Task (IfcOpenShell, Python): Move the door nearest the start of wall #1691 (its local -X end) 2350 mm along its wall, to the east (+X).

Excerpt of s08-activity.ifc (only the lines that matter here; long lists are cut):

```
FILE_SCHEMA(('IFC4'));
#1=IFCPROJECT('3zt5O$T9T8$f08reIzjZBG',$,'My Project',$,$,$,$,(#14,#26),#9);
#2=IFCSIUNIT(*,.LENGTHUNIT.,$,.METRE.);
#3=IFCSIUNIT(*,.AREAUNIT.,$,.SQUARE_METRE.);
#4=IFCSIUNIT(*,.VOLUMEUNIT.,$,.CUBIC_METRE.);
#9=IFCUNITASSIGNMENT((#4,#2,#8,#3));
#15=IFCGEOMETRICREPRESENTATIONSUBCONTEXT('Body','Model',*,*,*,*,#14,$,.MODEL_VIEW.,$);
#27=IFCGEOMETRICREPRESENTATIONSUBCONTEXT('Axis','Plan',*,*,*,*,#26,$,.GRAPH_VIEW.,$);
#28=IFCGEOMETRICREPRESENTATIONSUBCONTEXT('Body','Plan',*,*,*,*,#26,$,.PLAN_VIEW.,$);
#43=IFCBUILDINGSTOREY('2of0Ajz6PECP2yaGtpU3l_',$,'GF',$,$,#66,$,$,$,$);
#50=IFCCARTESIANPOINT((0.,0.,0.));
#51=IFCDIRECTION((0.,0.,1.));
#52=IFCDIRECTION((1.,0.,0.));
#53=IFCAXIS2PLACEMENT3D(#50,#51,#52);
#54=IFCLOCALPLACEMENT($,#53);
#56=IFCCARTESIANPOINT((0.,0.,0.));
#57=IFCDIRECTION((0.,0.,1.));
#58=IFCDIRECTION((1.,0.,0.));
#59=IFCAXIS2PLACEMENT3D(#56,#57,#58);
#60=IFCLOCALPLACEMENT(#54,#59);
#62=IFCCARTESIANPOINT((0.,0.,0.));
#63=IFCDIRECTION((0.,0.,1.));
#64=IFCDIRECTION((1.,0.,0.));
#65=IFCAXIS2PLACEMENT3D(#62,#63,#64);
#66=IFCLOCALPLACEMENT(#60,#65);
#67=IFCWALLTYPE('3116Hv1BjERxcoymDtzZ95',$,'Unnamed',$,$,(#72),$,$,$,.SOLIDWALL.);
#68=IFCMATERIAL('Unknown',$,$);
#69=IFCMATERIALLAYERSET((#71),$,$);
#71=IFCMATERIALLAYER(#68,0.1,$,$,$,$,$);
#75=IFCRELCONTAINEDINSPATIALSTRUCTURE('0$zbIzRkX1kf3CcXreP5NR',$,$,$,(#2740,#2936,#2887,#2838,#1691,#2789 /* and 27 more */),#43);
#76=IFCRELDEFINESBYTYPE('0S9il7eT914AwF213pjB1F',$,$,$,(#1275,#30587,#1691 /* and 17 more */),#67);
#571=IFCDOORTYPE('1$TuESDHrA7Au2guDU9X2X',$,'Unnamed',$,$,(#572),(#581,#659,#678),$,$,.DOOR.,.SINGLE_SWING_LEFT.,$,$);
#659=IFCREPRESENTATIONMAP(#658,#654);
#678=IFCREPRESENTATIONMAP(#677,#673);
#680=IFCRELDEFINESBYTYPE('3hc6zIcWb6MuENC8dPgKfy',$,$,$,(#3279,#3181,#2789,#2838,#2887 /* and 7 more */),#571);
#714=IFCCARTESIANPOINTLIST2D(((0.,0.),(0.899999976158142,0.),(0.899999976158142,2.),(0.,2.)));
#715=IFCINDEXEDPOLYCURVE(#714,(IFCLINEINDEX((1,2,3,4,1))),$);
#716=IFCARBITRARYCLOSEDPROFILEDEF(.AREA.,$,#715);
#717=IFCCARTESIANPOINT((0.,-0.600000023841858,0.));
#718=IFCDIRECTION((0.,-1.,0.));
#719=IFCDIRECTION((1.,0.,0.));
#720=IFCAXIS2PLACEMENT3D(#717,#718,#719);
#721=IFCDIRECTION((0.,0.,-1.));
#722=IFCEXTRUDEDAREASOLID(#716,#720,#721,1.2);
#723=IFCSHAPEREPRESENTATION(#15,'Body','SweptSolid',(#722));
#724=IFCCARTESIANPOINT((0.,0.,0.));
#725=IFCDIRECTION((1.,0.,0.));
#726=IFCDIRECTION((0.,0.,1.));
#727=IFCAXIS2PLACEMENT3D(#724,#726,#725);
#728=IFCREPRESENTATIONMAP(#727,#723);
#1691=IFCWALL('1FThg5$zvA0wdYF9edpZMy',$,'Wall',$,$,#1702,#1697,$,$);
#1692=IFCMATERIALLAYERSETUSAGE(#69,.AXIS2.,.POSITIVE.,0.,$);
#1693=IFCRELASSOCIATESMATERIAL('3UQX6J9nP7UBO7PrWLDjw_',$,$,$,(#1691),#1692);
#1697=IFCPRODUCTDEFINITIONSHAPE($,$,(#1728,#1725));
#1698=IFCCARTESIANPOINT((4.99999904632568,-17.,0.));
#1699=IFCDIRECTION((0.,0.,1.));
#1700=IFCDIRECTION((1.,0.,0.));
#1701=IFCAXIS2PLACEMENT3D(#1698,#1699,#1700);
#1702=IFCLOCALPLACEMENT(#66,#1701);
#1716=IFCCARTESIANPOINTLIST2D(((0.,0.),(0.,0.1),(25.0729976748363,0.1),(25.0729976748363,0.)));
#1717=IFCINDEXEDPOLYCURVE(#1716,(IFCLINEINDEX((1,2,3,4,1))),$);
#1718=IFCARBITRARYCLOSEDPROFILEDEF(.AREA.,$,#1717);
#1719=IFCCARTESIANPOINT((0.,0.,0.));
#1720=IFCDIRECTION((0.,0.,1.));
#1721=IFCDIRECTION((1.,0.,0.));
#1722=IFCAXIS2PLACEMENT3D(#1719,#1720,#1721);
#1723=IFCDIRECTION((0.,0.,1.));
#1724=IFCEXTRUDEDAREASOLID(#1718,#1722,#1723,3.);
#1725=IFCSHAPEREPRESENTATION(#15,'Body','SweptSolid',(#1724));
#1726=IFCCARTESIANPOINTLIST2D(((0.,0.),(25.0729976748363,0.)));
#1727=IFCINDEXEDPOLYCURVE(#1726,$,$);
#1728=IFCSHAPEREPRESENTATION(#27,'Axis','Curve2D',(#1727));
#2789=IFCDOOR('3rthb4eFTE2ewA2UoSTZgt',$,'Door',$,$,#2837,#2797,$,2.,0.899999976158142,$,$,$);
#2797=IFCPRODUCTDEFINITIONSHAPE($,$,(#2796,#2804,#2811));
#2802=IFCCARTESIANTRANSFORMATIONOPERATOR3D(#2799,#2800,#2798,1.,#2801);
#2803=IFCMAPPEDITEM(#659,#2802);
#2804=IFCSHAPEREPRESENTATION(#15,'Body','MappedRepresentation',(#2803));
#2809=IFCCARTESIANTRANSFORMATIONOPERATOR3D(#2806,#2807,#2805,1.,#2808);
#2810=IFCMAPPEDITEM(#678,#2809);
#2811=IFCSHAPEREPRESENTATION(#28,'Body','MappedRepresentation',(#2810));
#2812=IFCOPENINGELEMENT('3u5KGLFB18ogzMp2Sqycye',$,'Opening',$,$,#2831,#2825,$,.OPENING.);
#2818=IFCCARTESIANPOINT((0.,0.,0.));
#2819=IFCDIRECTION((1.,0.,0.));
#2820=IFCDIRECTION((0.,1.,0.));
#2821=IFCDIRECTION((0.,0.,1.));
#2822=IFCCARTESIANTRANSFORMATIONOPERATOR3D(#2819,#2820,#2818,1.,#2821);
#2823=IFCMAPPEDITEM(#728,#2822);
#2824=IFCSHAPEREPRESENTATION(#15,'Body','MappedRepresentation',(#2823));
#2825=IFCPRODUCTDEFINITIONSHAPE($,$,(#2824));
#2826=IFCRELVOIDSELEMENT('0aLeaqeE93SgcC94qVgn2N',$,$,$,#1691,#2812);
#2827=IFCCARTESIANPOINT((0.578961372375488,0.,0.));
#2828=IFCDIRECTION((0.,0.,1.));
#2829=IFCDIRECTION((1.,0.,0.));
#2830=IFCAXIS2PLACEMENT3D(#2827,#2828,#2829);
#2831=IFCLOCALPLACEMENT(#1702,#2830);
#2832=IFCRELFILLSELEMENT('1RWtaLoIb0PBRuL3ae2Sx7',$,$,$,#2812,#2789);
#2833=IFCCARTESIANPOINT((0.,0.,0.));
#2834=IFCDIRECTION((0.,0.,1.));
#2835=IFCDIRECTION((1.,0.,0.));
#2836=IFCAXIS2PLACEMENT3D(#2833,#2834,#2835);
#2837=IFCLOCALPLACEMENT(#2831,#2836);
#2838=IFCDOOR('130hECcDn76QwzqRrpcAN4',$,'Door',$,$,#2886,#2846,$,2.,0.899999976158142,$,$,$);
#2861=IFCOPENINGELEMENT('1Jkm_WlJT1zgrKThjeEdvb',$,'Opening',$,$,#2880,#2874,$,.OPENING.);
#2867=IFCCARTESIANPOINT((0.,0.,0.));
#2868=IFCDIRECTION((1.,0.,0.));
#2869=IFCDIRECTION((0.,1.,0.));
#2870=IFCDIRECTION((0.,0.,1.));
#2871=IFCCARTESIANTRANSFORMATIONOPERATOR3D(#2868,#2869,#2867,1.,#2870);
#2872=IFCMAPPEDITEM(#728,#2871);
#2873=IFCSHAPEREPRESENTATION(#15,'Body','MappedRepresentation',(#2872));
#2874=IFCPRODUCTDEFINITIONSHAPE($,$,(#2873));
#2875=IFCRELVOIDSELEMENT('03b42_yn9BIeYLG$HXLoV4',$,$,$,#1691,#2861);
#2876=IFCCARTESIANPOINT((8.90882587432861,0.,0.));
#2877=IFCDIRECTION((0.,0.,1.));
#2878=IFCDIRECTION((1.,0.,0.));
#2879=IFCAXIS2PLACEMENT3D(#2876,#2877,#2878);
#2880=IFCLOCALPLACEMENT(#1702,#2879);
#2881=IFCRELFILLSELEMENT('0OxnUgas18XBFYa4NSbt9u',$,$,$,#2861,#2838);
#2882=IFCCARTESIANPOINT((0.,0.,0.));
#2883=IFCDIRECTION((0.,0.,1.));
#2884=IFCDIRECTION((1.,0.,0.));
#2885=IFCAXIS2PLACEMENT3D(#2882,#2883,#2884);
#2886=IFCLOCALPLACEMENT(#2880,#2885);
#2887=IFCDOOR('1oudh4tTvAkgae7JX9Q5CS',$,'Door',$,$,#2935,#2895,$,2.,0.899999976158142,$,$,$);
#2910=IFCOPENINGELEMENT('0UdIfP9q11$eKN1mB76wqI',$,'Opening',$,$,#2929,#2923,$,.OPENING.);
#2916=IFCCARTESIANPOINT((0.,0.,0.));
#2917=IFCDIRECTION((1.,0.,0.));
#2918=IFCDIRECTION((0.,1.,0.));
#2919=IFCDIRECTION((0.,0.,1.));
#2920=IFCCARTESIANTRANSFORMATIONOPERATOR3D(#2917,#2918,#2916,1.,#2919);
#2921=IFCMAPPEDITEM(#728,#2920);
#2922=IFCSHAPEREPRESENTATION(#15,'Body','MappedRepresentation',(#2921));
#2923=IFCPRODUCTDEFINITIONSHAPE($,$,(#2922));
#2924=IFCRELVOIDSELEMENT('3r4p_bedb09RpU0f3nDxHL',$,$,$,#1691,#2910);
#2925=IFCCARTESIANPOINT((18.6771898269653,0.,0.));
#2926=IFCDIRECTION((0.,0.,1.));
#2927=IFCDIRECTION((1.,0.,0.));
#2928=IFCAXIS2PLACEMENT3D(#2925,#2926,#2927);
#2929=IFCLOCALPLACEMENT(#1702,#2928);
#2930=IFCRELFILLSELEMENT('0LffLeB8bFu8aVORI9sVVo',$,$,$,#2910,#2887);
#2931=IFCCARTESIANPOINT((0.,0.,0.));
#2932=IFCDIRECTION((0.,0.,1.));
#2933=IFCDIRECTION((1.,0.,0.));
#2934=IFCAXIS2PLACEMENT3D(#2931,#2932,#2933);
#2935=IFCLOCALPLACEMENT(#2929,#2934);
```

```python
import ifcopenshell
import ifcopenshell.api.geometry
import ifcopenshell.util.placement

model = ifcopenshell.open("s08-activity.ifc")

door = model.by_guid("3rthb4eFTE2ewA2UoSTZgt")
opening = door.FillsVoids[0].RelatingOpeningElement
wall = opening.VoidsElements[0].RelatingBuildingElement

wall_matrix = ifcopenshell.util.placement.get_local_placement(wall.ObjectPlacement)
shift = wall_matrix[:3, 0] * 2.35
before = ifcopenshell.util.placement.get_local_placement(door.ObjectPlacement)[:3, 3].copy()

# The door is placed relative to its opening, so it follows when the opening moves.
matrix = ifcopenshell.util.placement.get_local_placement(opening.ObjectPlacement)
matrix[:3, 3] += shift
ifcopenshell.api.geometry.edit_object_placement(
    model, product=opening, matrix=matrix, is_si=False, should_transform_children=True
)

after = ifcopenshell.util.placement.get_local_placement(door.ObjectPlacement)[:3, 3]
print("door moved by", (after - before).round(3) + 0.0)

model.write("s08-activity_v2.ifc")
```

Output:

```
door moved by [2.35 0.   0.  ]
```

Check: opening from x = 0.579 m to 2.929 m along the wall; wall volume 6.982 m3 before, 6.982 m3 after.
